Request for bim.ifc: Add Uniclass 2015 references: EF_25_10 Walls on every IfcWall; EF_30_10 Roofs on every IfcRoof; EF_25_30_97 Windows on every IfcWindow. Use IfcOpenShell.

First a look at what the model holds.

```python
import ifcopenshell

model = ifcopenshell.open("bim.ifc")
print(model.schema)
print("classifications:", [c.Name for c in model.by_type("IfcClassification")])
for ifc_class in ("IfcDoor", "IfcRoof", "IfcStair", "IfcWall", "IfcWindow"):
    print(ifc_class, len(model.by_type(ifc_class)))
```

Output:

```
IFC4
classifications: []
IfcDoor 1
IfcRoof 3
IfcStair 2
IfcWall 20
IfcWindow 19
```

```python
import ifcopenshell
import ifcopenshell.api.classification

model = ifcopenshell.open("bim.ifc")

system = ifcopenshell.api.classification.add_classification(model, classification="Uniclass 2015")

codes = {
    "IfcWall": ("EF_25_10", "Walls"),
    "IfcRoof": ("EF_30_10", "Roofs"),
    "IfcWindow": ("EF_25_30_97", "Windows"),
}
for ifc_class, (code, name) in codes.items():
    products = model.by_type(ifc_class)
    ifcopenshell.api.classification.add_reference(
        model, products=products, classification=system, identification=code, name=name
    )
    print(code, len(products))

model.write("bim_edited.ifc")
```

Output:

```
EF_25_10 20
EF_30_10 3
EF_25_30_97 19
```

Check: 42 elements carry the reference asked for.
